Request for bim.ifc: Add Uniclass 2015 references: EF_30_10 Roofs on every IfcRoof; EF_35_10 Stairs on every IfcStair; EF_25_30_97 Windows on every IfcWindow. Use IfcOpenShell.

First a look at what the model holds.

```python
import ifcopenshell

model = ifcopenshell.open("bim.ifc")
print(model.schema)
print("classifications:", [c.Name for c in model.by_type("IfcClassification")])
for ifc_class in ("IfcDoor", "IfcRoof", "IfcStair", "IfcWall", "IfcWindow"):
    print(ifc_class, len(model.by_type(ifc_class)))
```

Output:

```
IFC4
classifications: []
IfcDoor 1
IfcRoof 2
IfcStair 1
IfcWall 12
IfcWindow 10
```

```python
import ifcopenshell
import ifcopenshell.api.classification

model = ifcopenshell.open("bim.ifc")

system = ifcopenshell.api.classification.add_classification(model, classification="Uniclass 2015")

codes = {
    "IfcRoof": ("EF_30_10", "Roofs"),
    "IfcStair": ("EF_35_10", "Stairs"),
    "IfcWindow": ("EF_25_30_97", "Windows"),
}
for ifc_class, (code, name) in codes.items():
    products = model.by_type(ifc_class)
    ifcopenshell.api.classification.add_reference(
        model, products=products, classification=system, identification=code, name=name
    )
    print(code, len(products))

model.write("bim_updated.ifc")
```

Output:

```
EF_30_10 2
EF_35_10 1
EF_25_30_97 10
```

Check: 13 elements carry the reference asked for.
